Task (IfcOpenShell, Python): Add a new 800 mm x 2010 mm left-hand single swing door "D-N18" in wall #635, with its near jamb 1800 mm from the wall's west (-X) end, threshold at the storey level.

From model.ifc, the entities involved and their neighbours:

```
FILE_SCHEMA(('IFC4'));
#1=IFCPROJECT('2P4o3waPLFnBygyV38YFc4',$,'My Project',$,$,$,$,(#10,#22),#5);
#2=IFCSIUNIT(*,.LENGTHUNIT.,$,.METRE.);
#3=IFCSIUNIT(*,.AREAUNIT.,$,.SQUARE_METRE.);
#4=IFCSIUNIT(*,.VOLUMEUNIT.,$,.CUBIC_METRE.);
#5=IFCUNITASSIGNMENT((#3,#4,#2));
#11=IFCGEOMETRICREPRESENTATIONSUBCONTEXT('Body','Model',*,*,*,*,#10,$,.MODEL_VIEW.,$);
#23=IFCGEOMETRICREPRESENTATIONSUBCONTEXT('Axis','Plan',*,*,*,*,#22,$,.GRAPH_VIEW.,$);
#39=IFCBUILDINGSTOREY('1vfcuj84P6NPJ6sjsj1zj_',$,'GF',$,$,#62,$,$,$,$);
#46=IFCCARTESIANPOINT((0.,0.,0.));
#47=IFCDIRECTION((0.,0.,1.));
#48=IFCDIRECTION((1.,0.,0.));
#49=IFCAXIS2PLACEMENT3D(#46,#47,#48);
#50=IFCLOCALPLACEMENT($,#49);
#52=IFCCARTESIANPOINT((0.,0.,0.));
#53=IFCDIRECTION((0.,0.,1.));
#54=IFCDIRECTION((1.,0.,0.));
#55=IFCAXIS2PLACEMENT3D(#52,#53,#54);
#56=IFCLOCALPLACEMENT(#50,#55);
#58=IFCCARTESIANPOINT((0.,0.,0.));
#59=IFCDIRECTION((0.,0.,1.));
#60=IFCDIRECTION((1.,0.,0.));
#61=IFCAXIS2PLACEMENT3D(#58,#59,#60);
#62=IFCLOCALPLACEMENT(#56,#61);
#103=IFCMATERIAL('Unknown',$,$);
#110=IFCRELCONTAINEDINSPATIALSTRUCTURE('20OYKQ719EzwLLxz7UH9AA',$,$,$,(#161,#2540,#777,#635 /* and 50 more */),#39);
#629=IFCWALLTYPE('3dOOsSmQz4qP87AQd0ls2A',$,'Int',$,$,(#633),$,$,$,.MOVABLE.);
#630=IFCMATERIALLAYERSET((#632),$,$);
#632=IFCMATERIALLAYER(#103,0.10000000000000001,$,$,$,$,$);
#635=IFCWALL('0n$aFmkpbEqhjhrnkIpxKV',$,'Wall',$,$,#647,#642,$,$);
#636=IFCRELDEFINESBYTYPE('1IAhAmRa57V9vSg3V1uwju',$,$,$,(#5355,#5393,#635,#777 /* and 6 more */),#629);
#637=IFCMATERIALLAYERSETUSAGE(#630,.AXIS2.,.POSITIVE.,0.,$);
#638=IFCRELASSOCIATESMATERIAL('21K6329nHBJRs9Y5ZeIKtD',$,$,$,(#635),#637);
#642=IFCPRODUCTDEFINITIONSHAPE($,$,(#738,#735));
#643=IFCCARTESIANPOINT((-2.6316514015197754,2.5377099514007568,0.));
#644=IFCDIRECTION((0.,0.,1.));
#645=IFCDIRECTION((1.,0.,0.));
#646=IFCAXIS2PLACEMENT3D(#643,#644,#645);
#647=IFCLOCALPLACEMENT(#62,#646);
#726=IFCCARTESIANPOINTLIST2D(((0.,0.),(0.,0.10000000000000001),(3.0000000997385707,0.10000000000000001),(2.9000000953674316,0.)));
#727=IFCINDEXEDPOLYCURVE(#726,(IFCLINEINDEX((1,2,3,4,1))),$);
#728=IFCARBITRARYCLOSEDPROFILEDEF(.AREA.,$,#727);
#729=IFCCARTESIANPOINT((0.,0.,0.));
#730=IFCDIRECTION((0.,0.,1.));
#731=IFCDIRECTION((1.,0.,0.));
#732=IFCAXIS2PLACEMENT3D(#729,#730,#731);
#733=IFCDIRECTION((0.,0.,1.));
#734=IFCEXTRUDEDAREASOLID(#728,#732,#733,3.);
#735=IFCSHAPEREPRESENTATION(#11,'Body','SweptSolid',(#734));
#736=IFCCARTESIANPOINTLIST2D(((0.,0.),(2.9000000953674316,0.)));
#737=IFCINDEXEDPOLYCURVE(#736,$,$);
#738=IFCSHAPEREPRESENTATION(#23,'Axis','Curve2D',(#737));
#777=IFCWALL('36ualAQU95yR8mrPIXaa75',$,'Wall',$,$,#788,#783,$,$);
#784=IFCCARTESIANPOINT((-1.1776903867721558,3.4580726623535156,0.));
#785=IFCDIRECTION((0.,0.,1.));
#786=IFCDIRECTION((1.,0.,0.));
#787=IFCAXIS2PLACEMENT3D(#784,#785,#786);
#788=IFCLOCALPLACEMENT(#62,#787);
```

```python
import numpy as np
import ifcopenshell
import ifcopenshell.api.feature
import ifcopenshell.api.geometry
import ifcopenshell.api.root
import ifcopenshell.api.spatial
import ifcopenshell.geom
import ifcopenshell.util.element
import ifcopenshell.util.placement
import ifcopenshell.util.representation
import ifcopenshell.util.shape
import ifcopenshell.util.unit

model = ifcopenshell.open("model.ifc")
unit_scale = ifcopenshell.util.unit.calculate_unit_scale(model)
settings = ifcopenshell.geom.settings()


def volume(element):
    """Net volume in cubic metres, openings subtracted."""
    shape = ifcopenshell.geom.create_shape(settings, element)
    return ifcopenshell.util.shape.get_volume(shape.geometry)


wall = model.by_guid("0n$aFmkpbEqhjhrnkIpxKV")
storey = ifcopenshell.util.element.get_container(wall, ifc_class="IfcBuildingStorey")
context = ifcopenshell.util.representation.get_context(model, "Model", "Body", "MODEL_VIEW")
before = volume(wall)

width, height, from_end, sill = 0.8, 2.01, 1.8, 0.0  # metres

# The wall runs along its own X axis, and the end named is its -X end.
wall_shape = ifcopenshell.geom.create_shape(settings, wall)
x, y, z = ifcopenshell.util.shape.get_vertices(wall_shape.geometry).T
start = x.min() + from_end
face, thickness = float(y.min()), float(y.max() - y.min())
wall_matrix = ifcopenshell.util.placement.get_local_placement(wall.ObjectPlacement)
level = ifcopenshell.util.placement.get_local_placement(storey.ObjectPlacement)[2, 3]


def in_wall(x, y):
    """Placement at x, y metres in the wall's axes, at sill height."""
    matrix = wall_matrix.copy()
    matrix[:, 3] = wall_matrix @ np.array([x / unit_scale, y / unit_scale, 0.0, 1.0])
    matrix[2, 3] = level + sill / unit_scale
    return matrix


# Opening: a box that overshoots both wall faces by 50 mm.
opening = ifcopenshell.api.root.create_entity(model, ifc_class="IfcOpeningElement", predefined_type="OPENING")
box = ifcopenshell.api.geometry.add_wall_representation(
    model, context=context, length=width, height=height, thickness=thickness + 0.1
)
ifcopenshell.api.geometry.assign_representation(model, product=opening, representation=box)
ifcopenshell.api.geometry.edit_object_placement(model, product=opening, matrix=in_wall(start, face - 0.05), is_si=False)
ifcopenshell.api.feature.add_feature(model, feature=opening, element=wall)

door = ifcopenshell.api.root.create_entity(model, ifc_class="IfcDoor", name="D-N18", predefined_type="DOOR")
door.OverallWidth, door.OverallHeight = width / unit_scale, height / unit_scale
door.OperationType = "SINGLE_SWING_LEFT"
body = ifcopenshell.api.geometry.add_door_representation(
    model,
    context=context,
    overall_width=door.OverallWidth,
    overall_height=door.OverallHeight,
    operation_type="SINGLE_SWING_LEFT",
    lining_properties={"LiningDepth": thickness / unit_scale, "ThresholdDepth": thickness / unit_scale},
)
ifcopenshell.api.geometry.assign_representation(model, product=door, representation=body)
ifcopenshell.api.spatial.assign_container(model, products=[door], relating_structure=storey)
ifcopenshell.api.feature.add_filling(model, opening=opening, element=door)

# The lining spans the wall, so the door starts at the wall face.
ifcopenshell.api.geometry.edit_object_placement(model, product=door, matrix=in_wall(start, face), is_si=False)

after = volume(wall)

print(f"wall volume {before:.3f} -> {after:.3f} m3")

model.write("model_updated.ifc")
```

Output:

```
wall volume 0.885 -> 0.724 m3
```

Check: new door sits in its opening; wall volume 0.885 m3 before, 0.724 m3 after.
